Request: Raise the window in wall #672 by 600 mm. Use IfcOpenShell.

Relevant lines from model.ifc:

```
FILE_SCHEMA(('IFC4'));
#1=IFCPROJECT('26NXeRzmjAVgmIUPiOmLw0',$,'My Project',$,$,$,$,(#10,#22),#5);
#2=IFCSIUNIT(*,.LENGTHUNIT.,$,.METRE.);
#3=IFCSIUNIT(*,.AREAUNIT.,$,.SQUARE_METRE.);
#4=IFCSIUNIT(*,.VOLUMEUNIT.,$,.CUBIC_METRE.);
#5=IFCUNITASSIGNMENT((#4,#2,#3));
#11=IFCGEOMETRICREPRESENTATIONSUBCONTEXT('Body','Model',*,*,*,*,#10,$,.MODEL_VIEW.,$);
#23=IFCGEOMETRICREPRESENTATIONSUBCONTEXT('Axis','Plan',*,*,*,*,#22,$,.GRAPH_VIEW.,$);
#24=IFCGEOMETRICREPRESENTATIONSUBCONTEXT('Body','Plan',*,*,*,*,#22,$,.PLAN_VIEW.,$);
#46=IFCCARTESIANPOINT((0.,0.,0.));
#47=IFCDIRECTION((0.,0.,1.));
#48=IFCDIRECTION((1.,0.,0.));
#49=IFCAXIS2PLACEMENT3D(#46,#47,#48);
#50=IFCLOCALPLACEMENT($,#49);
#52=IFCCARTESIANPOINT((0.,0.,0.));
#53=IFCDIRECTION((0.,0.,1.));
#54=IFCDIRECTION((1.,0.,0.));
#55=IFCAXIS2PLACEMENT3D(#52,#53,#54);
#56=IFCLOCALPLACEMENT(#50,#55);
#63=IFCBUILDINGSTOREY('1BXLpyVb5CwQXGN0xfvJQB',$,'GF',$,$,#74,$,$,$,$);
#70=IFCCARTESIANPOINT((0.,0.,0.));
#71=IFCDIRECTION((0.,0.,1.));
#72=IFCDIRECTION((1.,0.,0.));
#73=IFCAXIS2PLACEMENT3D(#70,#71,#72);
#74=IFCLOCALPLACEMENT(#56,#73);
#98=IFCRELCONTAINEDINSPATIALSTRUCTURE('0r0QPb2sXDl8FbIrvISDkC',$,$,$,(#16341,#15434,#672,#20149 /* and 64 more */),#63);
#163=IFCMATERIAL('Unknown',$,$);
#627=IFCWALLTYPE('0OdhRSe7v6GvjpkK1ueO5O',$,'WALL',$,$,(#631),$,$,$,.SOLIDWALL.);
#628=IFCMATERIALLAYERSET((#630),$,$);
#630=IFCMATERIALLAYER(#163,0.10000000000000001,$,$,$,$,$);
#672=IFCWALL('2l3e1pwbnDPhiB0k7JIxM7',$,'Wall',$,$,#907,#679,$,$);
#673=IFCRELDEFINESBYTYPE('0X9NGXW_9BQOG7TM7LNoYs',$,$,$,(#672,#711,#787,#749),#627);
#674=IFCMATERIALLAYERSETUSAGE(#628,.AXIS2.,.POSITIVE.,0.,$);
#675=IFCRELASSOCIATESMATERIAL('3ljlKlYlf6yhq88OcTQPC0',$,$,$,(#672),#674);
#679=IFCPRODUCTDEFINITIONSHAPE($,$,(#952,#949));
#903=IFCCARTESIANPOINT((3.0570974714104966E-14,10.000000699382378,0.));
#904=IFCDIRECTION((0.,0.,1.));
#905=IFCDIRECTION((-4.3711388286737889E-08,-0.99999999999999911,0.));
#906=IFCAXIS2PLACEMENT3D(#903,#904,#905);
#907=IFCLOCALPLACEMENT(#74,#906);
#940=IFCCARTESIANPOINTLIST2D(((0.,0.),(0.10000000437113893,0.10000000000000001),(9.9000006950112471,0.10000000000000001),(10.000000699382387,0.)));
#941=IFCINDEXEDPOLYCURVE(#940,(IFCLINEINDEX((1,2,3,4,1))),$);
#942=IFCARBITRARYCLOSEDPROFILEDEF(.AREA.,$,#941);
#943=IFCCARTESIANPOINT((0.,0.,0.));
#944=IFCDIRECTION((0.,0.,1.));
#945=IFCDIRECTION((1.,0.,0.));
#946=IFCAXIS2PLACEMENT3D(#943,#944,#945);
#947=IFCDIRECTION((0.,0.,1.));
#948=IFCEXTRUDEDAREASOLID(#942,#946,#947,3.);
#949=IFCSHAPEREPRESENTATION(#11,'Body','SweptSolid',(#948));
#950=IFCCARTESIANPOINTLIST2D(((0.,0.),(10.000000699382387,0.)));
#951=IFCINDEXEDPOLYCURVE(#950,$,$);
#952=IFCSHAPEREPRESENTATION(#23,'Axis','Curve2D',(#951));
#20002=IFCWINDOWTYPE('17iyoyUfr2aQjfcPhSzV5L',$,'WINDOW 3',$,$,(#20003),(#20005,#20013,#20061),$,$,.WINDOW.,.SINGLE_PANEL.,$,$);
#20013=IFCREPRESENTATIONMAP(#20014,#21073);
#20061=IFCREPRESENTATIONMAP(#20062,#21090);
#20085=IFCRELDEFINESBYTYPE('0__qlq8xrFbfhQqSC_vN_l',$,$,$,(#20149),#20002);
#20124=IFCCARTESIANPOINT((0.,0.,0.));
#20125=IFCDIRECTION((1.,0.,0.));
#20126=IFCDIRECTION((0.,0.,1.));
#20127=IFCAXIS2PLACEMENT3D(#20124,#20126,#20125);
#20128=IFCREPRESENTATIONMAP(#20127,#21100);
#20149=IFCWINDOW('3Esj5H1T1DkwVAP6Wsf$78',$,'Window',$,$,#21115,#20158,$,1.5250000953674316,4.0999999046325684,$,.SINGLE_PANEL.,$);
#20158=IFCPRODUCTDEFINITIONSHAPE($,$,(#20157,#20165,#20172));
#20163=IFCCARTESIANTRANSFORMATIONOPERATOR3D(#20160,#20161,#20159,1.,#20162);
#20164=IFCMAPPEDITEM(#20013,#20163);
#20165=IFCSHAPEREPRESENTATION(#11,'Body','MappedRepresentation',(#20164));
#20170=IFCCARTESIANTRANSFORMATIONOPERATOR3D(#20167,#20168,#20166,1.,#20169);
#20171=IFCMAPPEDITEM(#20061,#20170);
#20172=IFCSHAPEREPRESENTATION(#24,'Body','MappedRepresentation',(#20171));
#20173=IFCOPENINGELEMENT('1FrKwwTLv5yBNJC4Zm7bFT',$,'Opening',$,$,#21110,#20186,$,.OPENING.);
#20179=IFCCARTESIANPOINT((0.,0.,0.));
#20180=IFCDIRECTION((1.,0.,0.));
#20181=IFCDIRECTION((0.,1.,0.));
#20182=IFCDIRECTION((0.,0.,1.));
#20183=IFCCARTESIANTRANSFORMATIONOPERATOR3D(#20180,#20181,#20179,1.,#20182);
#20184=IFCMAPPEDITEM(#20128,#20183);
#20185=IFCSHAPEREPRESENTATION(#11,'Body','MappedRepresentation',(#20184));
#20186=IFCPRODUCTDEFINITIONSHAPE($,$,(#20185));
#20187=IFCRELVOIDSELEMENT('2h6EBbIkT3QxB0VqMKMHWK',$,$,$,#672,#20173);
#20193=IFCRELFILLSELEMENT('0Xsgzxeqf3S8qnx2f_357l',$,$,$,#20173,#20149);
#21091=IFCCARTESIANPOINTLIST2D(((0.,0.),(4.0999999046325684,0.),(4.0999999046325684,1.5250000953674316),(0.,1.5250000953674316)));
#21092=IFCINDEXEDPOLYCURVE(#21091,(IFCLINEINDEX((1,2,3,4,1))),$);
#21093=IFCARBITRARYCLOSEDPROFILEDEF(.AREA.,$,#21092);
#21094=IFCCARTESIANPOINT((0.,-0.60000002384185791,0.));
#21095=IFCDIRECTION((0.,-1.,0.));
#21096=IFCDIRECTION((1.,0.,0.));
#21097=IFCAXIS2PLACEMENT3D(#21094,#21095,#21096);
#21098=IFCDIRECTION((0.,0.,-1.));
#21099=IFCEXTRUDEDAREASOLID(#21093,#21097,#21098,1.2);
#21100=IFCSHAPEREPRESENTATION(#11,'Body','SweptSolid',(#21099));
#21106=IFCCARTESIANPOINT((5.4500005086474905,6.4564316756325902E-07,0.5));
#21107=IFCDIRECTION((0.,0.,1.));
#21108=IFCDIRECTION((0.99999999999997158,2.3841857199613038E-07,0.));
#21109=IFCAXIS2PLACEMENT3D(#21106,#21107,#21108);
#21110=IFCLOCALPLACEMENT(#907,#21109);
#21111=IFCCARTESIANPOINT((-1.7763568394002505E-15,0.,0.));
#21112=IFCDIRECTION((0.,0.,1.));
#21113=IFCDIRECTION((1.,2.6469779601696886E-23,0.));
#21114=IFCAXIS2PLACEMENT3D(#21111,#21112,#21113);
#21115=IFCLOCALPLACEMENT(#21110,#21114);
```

```python
import numpy as np
import ifcopenshell
import ifcopenshell.api.geometry
import ifcopenshell.util.placement
import ifcopenshell.util.unit

model = ifcopenshell.open("model.ifc")
unit_scale = ifcopenshell.util.unit.calculate_unit_scale(model)

window = model.by_guid("3Esj5H1T1DkwVAP6Wsf$78")
opening = window.FillsVoids[0].RelatingOpeningElement
dz = 0.6

shift = np.array([0.0, 0.0, dz])
# The window is placed relative to its opening, so it follows when the opening moves.
matrix = ifcopenshell.util.placement.get_local_placement(opening.ObjectPlacement)
matrix[:3, 3] += shift
ifcopenshell.api.geometry.edit_object_placement(
    model, product=opening, matrix=matrix, is_si=False, should_transform_children=True
)

print(f"moved by {dz * unit_scale:+.3f} m")

model.write("model-out.ifc")
```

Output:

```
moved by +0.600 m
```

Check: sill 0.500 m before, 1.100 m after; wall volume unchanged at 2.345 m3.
